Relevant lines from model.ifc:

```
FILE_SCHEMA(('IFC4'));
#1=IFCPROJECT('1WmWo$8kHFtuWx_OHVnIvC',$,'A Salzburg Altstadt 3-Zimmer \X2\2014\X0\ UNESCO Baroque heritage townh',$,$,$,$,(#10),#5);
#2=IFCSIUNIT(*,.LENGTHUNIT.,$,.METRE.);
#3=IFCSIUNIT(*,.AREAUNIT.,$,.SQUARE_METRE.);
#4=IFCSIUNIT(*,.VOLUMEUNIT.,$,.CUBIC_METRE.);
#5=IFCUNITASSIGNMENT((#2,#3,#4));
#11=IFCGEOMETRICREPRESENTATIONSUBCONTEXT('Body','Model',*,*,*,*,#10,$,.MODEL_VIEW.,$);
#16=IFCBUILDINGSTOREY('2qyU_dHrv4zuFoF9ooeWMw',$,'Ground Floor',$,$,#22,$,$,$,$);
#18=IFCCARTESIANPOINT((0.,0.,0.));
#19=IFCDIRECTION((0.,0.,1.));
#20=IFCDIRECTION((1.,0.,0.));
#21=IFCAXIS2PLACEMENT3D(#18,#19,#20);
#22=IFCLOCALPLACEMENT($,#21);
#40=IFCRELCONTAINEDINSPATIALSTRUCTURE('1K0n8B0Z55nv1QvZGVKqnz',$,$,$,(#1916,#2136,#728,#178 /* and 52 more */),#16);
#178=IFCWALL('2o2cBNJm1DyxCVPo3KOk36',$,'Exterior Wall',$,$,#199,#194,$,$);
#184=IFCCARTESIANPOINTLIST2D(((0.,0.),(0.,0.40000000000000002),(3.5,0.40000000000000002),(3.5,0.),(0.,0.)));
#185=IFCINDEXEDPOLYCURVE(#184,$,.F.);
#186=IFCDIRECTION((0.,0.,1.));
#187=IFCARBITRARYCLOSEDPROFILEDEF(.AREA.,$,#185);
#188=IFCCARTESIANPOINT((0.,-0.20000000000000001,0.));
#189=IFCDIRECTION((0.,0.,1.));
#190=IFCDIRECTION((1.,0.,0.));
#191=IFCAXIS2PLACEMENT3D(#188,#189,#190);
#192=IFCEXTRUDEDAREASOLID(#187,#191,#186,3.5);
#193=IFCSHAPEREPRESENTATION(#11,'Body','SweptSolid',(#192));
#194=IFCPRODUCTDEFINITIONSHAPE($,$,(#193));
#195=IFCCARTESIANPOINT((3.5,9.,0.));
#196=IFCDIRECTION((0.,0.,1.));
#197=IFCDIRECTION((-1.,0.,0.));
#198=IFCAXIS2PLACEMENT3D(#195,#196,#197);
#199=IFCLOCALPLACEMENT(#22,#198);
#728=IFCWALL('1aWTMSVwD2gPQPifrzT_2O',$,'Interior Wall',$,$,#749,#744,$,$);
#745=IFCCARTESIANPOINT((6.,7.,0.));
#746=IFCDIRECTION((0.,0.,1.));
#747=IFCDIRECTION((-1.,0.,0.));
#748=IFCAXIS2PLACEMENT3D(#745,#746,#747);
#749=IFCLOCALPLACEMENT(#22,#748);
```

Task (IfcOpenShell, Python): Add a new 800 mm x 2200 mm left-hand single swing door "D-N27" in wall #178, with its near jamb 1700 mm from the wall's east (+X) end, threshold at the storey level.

```python
import numpy as np
import ifcopenshell
import ifcopenshell.api.feature
import ifcopenshell.api.geometry
import ifcopenshell.api.root
import ifcopenshell.api.spatial
import ifcopenshell.geom
import ifcopenshell.util.element
import ifcopenshell.util.placement
import ifcopenshell.util.representation
import ifcopenshell.util.shape
import ifcopenshell.util.unit

model = ifcopenshell.open("model.ifc")
unit_scale = ifcopenshell.util.unit.calculate_unit_scale(model)
settings = ifcopenshell.geom.settings()


def volume(element):
    """Net volume in cubic metres, openings subtracted."""
    shape = ifcopenshell.geom.create_shape(settings, element)
    return ifcopenshell.util.shape.get_volume(shape.geometry)


wall = model.by_id(178)
storey = ifcopenshell.util.element.get_container(wall, ifc_class="IfcBuildingStorey")
context = ifcopenshell.util.representation.get_context(model, "Model", "Body", "MODEL_VIEW")
before = volume(wall)

width, height, from_end, sill = 0.8, 2.2, 1.7, 0.0  # metres

# The wall runs along its own X axis, and the end named is its -X end.
wall_shape = ifcopenshell.geom.create_shape(settings, wall)
x, y, z = ifcopenshell.util.shape.get_vertices(wall_shape.geometry).T
start = x.min() + from_end
face, thickness = float(y.min()), float(y.max() - y.min())
wall_matrix = ifcopenshell.util.placement.get_local_placement(wall.ObjectPlacement)
level = ifcopenshell.util.placement.get_local_placement(storey.ObjectPlacement)[2, 3]


def in_wall(x, y):
    """Placement at x, y metres in the wall's axes, at sill height."""
    matrix = wall_matrix.copy()
    matrix[:, 3] = wall_matrix @ np.array([x / unit_scale, y / unit_scale, 0.0, 1.0])
    matrix[2, 3] = level + sill / unit_scale
    return matrix


# Opening: a box that overshoots both wall faces by 50 mm.
opening = ifcopenshell.api.root.create_entity(model, ifc_class="IfcOpeningElement", predefined_type="OPENING")
box = ifcopenshell.api.geometry.add_wall_representation(
    model, context=context, length=width, height=height, thickness=thickness + 0.1
)
ifcopenshell.api.geometry.assign_representation(model, product=opening, representation=box)
ifcopenshell.api.geometry.edit_object_placement(model, product=opening, matrix=in_wall(start, face - 0.05), is_si=False)
ifcopenshell.api.feature.add_feature(model, feature=opening, element=wall)

door = ifcopenshell.api.root.create_entity(model, ifc_class="IfcDoor", name="D-N27", predefined_type="DOOR")
door.OverallWidth, door.OverallHeight = width / unit_scale, height / unit_scale
door.OperationType = "SINGLE_SWING_LEFT"
body = ifcopenshell.api.geometry.add_door_representation(
    model,
    context=context,
    overall_width=door.OverallWidth,
    overall_height=door.OverallHeight,
    operation_type="SINGLE_SWING_LEFT",
    lining_properties={"LiningDepth": thickness / unit_scale, "ThresholdDepth": thickness / unit_scale},
)
ifcopenshell.api.geometry.assign_representation(model, product=door, representation=body)
ifcopenshell.api.spatial.assign_container(model, products=[door], relating_structure=storey)
ifcopenshell.api.feature.add_filling(model, opening=opening, element=door)

# The lining spans the wall, so the door starts at the wall face.
ifcopenshell.api.geometry.edit_object_placement(model, product=door, matrix=in_wall(start, face), is_si=False)

after = volume(wall)

print(f"wall volume {before:.3f} -> {after:.3f} m3")

model.write("model_v2.ifc")
```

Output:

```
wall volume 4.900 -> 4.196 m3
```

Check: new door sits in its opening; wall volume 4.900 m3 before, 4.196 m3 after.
